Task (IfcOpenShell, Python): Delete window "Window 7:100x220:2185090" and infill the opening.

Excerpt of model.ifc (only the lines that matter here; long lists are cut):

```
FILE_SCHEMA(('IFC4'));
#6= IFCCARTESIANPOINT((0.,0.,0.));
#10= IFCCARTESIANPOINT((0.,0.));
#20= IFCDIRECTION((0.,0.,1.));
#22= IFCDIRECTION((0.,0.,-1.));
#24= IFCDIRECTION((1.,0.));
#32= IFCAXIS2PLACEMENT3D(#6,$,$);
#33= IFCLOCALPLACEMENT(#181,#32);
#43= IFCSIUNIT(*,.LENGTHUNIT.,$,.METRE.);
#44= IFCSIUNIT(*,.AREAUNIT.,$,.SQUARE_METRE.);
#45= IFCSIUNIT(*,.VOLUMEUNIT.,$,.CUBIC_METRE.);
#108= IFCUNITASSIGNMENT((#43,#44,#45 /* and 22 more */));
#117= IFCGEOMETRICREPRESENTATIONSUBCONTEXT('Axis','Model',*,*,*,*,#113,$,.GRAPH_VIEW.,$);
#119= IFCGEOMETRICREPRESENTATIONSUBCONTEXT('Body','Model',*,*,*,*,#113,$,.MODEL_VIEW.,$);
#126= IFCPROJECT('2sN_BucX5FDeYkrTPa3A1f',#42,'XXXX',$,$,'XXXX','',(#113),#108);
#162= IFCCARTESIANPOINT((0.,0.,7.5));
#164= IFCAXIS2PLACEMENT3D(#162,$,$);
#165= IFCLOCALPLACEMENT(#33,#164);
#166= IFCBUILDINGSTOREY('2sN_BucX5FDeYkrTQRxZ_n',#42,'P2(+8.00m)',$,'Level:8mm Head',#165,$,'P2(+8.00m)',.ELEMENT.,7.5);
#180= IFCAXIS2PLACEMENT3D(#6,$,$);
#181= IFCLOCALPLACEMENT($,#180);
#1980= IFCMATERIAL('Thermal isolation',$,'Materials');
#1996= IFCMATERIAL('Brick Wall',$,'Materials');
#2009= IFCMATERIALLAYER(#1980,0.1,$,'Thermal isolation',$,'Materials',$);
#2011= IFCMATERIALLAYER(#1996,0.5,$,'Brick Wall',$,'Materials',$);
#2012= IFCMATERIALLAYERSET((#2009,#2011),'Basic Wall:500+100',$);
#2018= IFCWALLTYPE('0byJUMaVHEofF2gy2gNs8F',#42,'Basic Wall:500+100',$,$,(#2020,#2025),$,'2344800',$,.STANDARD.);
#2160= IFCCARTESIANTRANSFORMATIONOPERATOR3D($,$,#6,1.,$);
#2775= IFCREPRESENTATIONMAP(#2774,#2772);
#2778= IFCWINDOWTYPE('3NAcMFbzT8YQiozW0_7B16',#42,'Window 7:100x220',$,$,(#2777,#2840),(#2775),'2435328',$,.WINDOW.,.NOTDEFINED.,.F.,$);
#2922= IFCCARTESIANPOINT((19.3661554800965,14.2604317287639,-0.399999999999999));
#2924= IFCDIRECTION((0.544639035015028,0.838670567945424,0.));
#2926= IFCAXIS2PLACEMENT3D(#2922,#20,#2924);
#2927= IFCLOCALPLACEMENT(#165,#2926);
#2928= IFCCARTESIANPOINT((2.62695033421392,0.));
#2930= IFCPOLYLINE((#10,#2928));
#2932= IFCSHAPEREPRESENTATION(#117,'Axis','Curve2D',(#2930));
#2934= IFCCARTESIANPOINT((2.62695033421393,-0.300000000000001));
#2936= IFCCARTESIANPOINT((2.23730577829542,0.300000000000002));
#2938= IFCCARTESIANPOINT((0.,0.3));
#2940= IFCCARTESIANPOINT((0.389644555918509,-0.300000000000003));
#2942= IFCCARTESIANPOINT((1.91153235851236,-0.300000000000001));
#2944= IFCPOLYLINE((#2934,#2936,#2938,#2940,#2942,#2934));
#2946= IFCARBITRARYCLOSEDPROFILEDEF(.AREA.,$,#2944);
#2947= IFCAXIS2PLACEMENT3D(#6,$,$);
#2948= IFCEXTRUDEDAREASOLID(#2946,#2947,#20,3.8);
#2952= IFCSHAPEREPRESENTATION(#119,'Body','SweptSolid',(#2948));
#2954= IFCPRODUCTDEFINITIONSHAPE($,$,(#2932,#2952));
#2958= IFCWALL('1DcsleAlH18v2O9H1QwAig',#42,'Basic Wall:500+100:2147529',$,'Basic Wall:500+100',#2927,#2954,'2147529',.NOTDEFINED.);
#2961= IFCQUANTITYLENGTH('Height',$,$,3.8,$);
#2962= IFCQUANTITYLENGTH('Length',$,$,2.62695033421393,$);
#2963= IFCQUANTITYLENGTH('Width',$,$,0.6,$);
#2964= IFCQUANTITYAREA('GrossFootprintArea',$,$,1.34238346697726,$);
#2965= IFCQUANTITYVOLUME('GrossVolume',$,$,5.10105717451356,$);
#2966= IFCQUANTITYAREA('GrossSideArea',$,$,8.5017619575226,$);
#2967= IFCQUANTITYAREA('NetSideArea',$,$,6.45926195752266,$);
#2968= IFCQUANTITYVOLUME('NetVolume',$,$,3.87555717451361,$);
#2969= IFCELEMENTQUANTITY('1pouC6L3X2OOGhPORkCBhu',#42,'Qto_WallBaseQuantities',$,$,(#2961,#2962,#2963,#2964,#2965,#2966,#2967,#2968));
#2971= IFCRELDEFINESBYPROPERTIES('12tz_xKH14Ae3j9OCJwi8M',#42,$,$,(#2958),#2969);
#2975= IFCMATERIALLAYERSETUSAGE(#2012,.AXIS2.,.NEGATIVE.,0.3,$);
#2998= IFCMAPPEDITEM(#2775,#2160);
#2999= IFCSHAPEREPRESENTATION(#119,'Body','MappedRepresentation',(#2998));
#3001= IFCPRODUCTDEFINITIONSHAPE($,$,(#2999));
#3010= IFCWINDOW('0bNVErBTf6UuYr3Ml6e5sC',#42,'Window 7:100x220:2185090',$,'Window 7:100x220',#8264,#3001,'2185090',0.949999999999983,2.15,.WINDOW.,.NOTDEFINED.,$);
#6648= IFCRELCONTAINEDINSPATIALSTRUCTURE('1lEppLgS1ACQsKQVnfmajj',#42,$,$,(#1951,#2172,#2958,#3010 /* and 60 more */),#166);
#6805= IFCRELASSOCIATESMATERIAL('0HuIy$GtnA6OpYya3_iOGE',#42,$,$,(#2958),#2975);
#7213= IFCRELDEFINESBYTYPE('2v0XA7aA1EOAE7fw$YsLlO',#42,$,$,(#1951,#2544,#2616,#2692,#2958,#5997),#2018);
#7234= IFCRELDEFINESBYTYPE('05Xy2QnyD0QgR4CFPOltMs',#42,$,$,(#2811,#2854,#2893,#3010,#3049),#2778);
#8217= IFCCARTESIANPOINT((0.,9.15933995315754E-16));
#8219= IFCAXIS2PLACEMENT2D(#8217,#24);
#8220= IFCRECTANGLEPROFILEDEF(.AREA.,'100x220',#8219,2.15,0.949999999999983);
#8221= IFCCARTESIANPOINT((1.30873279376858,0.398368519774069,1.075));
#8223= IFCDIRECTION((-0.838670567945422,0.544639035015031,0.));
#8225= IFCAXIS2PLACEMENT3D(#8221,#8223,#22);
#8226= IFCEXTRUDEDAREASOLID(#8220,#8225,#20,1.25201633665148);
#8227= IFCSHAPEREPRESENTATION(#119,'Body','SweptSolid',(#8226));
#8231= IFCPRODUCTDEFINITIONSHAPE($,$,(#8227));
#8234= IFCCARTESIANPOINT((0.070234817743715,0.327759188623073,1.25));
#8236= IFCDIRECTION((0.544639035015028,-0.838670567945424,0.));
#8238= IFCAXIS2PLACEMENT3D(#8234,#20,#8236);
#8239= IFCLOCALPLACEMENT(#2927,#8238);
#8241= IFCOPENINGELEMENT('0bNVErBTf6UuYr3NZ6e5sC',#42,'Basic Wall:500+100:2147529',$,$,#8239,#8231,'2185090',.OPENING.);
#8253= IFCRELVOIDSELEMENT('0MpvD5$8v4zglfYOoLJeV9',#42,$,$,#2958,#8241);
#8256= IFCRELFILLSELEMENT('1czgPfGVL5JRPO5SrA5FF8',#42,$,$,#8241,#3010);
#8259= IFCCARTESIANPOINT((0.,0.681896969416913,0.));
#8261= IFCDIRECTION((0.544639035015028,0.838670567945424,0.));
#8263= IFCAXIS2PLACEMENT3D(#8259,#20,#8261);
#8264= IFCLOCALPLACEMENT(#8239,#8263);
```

```python
import ifcopenshell
import ifcopenshell.api.feature
import ifcopenshell.api.pset
import ifcopenshell.api.root
import ifcopenshell.geom
import ifcopenshell.util.element
import ifcopenshell.util.shape
import ifcopenshell.util.unit

model = ifcopenshell.open("model.ifc")
area_scale = ifcopenshell.util.unit.calculate_unit_scale(model, "AREAUNIT")
volume_scale = ifcopenshell.util.unit.calculate_unit_scale(model, "VOLUMEUNIT")
settings = ifcopenshell.geom.settings()


def volume(element):
    """Net volume in cubic metres, openings subtracted."""
    shape = ifcopenshell.geom.create_shape(settings, element)
    return ifcopenshell.util.shape.get_volume(shape.geometry)


window = model.by_id(3010)
opening = window.FillsVoids[0].RelatingOpeningElement
wall = opening.VoidsElements[0].RelatingBuildingElement
before = volume(wall)

ifcopenshell.api.root.remove_product(model, product=window)
ifcopenshell.api.feature.remove_feature(model, feature=opening)

after = volume(wall)
thickness = 0.6  # wall thickness in metres

# Update the wall's stored quantities.
qto = model.by_id(ifcopenshell.util.element.get_pset(wall, "Qto_WallBaseQuantities", should_inherit=False)["id"])
ifcopenshell.api.pset.edit_qto(model, qto=qto, properties={
    "NetSideArea": after / thickness / area_scale,
    "NetVolume": after / volume_scale,
})

print(f"wall volume {before:.3f} -> {after:.3f} m3")

model.write("model_rev.ifc")
```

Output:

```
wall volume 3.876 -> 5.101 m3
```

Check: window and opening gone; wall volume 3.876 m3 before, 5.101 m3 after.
